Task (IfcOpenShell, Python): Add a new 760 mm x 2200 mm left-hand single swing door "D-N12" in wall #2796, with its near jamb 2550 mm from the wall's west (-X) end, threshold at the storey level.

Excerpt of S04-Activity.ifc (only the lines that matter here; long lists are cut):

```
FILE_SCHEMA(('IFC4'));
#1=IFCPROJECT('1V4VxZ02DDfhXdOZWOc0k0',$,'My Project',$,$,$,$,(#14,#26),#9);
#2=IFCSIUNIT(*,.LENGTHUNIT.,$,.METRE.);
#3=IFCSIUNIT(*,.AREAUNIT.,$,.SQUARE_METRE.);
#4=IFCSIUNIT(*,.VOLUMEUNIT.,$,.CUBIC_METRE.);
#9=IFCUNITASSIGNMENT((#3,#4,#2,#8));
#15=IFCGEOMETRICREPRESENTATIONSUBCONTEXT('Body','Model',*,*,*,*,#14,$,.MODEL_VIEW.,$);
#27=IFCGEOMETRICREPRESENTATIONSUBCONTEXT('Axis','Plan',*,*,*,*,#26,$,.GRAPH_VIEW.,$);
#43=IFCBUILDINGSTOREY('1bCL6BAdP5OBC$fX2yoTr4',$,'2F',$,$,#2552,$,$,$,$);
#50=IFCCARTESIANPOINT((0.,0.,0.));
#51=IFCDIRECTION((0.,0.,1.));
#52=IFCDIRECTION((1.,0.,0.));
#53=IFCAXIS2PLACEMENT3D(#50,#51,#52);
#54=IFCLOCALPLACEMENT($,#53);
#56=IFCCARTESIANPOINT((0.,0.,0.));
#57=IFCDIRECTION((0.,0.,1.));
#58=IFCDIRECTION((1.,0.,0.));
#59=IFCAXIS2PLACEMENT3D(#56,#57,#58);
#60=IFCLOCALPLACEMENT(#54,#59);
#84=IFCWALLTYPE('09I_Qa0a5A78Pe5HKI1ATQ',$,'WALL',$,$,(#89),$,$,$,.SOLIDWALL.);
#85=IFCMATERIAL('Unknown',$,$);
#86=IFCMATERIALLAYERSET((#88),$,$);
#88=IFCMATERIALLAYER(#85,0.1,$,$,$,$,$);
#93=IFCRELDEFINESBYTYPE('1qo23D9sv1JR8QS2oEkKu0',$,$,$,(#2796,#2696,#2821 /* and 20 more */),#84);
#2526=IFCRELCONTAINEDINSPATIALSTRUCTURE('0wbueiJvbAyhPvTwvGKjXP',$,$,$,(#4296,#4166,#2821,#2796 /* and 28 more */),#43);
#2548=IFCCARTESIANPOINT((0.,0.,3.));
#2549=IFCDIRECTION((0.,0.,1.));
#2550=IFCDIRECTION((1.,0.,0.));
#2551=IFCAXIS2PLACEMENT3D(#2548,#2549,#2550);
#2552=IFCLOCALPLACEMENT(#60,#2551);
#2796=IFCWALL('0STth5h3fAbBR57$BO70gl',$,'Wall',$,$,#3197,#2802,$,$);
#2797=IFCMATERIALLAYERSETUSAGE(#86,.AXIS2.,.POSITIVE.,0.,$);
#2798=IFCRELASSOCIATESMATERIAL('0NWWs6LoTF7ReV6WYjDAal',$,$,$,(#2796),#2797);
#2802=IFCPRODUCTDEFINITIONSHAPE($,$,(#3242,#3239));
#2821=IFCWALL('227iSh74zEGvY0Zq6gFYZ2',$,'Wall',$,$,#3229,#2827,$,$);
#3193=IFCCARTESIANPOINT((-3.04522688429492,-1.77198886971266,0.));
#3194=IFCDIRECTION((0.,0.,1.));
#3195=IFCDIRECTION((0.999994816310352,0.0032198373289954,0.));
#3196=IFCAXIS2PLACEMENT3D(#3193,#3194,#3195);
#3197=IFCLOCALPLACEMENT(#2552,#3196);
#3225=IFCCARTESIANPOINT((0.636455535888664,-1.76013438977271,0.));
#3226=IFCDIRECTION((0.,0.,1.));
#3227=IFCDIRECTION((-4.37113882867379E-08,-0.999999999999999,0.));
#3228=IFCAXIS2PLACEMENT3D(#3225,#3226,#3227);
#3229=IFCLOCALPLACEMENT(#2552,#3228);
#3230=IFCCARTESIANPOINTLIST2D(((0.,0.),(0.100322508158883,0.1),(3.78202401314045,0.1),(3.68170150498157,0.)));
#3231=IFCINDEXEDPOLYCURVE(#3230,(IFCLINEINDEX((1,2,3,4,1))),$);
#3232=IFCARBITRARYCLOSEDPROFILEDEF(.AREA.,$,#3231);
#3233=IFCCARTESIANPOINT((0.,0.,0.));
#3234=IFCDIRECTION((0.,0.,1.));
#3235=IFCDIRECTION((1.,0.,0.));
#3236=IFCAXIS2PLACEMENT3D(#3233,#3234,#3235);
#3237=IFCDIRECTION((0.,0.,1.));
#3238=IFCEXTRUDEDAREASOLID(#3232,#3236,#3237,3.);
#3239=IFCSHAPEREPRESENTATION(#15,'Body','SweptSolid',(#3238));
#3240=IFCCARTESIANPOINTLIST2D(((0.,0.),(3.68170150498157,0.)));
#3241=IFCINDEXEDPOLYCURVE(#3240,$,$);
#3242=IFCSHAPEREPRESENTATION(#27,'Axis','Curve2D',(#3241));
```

```python
import numpy as np
import ifcopenshell
import ifcopenshell.api.feature
import ifcopenshell.api.geometry
import ifcopenshell.api.root
import ifcopenshell.api.spatial
import ifcopenshell.geom
import ifcopenshell.util.element
import ifcopenshell.util.placement
import ifcopenshell.util.representation
import ifcopenshell.util.shape
import ifcopenshell.util.unit

model = ifcopenshell.open("S04-Activity.ifc")
unit_scale = ifcopenshell.util.unit.calculate_unit_scale(model)
settings = ifcopenshell.geom.settings()


def volume(element):
    """Net volume in cubic metres, openings subtracted."""
    shape = ifcopenshell.geom.create_shape(settings, element)
    return ifcopenshell.util.shape.get_volume(shape.geometry)


wall = model.by_guid("0STth5h3fAbBR57$BO70gl")
storey = ifcopenshell.util.element.get_container(wall, ifc_class="IfcBuildingStorey")
context = ifcopenshell.util.representation.get_context(model, "Model", "Body", "MODEL_VIEW")
before = volume(wall)

width, height, from_end, sill = 0.76, 2.2, 2.55, 0.0  # metres

# The wall runs along its own X axis, and the end named is its -X end.
wall_shape = ifcopenshell.geom.create_shape(settings, wall)
x, y, z = ifcopenshell.util.shape.get_vertices(wall_shape.geometry).T
start = x.min() + from_end
face, thickness = float(y.min()), float(y.max() - y.min())
wall_matrix = ifcopenshell.util.placement.get_local_placement(wall.ObjectPlacement)
level = ifcopenshell.util.placement.get_local_placement(storey.ObjectPlacement)[2, 3]


def in_wall(x, y):
    """Placement at x, y metres in the wall's axes, at sill height."""
    matrix = wall_matrix.copy()
    matrix[:, 3] = wall_matrix @ np.array([x / unit_scale, y / unit_scale, 0.0, 1.0])
    matrix[2, 3] = level + sill / unit_scale
    return matrix


# Opening: a box that overshoots both wall faces by 50 mm.
opening = ifcopenshell.api.root.create_entity(model, ifc_class="IfcOpeningElement", predefined_type="OPENING")
box = ifcopenshell.api.geometry.add_wall_representation(
    model, context=context, length=width, height=height, thickness=thickness + 0.1
)
ifcopenshell.api.geometry.assign_representation(model, product=opening, representation=box)
ifcopenshell.api.geometry.edit_object_placement(model, product=opening, matrix=in_wall(start, face - 0.05), is_si=False)
ifcopenshell.api.feature.add_feature(model, feature=opening, element=wall)

door = ifcopenshell.api.root.create_entity(model, ifc_class="IfcDoor", name="D-N12", predefined_type="DOOR")
door.OverallWidth, door.OverallHeight = width / unit_scale, height / unit_scale
door.OperationType = "SINGLE_SWING_LEFT"
body = ifcopenshell.api.geometry.add_door_representation(
    model,
    context=context,
    overall_width=door.OverallWidth,
    overall_height=door.OverallHeight,
    operation_type="SINGLE_SWING_LEFT",
    lining_properties={"LiningDepth": thickness / unit_scale, "ThresholdDepth": thickness / unit_scale},
)
ifcopenshell.api.geometry.assign_representation(model, product=door, representation=body)
ifcopenshell.api.spatial.assign_container(model, products=[door], relating_structure=storey)
ifcopenshell.api.feature.add_filling(model, opening=opening, element=door)

# The lining spans the wall, so the door starts at the wall face.
ifcopenshell.api.geometry.edit_object_placement(model, product=door, matrix=in_wall(start, face), is_si=False)

after = volume(wall)

print(f"wall volume {before:.3f} -> {after:.3f} m3")

model.write("S04-Activity_edited.ifc")
```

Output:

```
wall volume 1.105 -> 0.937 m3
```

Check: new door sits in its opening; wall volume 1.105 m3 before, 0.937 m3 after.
